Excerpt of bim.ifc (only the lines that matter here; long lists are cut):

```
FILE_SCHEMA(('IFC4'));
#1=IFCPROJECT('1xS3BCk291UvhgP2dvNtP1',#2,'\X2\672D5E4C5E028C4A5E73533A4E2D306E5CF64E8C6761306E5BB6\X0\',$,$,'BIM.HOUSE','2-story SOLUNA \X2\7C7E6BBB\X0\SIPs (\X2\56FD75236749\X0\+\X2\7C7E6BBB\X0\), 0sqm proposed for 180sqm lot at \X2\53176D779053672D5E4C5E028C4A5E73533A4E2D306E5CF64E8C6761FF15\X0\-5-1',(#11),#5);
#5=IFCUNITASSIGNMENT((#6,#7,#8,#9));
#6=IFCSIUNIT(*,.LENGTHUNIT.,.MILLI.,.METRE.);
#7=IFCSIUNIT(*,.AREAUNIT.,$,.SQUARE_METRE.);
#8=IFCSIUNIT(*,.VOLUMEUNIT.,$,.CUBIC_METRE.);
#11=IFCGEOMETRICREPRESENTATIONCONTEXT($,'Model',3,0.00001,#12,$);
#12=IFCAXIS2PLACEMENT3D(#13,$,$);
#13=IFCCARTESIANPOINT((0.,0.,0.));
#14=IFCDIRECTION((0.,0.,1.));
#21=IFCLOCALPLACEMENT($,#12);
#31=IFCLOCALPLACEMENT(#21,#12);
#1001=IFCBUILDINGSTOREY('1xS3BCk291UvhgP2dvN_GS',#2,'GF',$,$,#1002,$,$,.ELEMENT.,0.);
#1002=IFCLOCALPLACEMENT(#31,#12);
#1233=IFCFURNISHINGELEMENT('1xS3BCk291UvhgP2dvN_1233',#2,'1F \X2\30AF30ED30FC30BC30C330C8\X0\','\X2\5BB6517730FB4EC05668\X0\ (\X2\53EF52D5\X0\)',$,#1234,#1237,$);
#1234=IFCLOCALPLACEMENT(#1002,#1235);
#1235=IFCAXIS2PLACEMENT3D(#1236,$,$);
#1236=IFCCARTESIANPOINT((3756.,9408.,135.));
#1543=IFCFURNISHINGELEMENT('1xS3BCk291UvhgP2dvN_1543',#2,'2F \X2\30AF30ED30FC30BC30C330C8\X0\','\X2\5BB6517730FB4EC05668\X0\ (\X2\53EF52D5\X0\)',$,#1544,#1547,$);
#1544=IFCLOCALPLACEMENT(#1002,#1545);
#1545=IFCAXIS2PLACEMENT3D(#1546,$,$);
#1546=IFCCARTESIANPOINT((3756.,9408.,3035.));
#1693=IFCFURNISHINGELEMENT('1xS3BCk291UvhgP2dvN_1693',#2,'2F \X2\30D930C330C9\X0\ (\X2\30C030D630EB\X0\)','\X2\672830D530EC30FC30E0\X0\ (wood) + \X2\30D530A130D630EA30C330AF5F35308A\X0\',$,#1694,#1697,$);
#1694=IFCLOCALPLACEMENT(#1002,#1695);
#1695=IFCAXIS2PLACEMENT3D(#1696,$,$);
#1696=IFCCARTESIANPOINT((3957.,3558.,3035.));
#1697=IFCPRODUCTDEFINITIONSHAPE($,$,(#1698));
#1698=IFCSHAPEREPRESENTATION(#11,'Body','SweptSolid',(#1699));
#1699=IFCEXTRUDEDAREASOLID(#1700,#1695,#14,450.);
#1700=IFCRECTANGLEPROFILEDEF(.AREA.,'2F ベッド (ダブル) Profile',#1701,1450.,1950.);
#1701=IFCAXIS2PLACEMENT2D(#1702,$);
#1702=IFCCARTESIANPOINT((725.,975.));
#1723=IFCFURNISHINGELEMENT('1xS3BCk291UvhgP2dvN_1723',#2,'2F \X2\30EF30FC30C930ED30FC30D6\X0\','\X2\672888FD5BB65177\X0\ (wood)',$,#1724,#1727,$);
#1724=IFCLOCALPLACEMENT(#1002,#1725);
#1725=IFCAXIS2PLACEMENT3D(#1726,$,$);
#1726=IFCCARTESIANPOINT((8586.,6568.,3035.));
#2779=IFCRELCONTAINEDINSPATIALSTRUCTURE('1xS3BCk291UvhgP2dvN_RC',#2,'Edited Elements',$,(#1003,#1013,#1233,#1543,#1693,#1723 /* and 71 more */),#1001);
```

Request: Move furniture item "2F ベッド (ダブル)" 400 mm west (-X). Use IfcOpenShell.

```python
import ifcopenshell
import ifcopenshell.api.geometry
import ifcopenshell.util.placement
import ifcopenshell.util.unit

model = ifcopenshell.open("bim.ifc")
unit_scale = ifcopenshell.util.unit.calculate_unit_scale(model)

item = model.by_guid("1xS3BCk291UvhgP2dvN_1693")
matrix = ifcopenshell.util.placement.get_local_placement(item.ObjectPlacement)
matrix[0, 3] -= 0.4 / unit_scale
ifcopenshell.api.geometry.edit_object_placement(model, product=item, matrix=matrix, is_si=False)

print(ifcopenshell.util.placement.get_local_placement(item.ObjectPlacement).round(3) + 0.0)

model.write("bim_edited.ifc")
```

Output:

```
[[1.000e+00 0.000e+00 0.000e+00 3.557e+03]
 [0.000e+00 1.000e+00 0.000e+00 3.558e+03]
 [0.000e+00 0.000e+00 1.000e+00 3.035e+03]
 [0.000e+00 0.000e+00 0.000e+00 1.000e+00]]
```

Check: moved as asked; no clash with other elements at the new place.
